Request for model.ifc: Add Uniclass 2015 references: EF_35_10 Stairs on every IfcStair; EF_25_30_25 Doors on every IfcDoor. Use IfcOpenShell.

First a look at what the model holds.

```python
import ifcopenshell

model = ifcopenshell.open("model.ifc")
print(model.schema)
print("classifications:", [c.Name for c in model.by_type("IfcClassification")])
for ifc_class in ("IfcDoor", "IfcRoof", "IfcStair", "IfcWall", "IfcWindow"):
    print(ifc_class, len(model.by_type(ifc_class)))
```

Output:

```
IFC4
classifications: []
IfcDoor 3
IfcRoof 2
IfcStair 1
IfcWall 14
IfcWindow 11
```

```python
import ifcopenshell
import ifcopenshell.api.classification

model = ifcopenshell.open("model.ifc")

system = ifcopenshell.api.classification.add_classification(model, classification="Uniclass 2015")

codes = {
    "IfcStair": ("EF_35_10", "Stairs"),
    "IfcDoor": ("EF_25_30_25", "Doors"),
}
for ifc_class, (code, name) in codes.items():
    products = model.by_type(ifc_class)
    ifcopenshell.api.classification.add_reference(
        model, products=products, classification=system, identification=code, name=name
    )
    print(code, len(products))

model.write("model_edited.ifc")
```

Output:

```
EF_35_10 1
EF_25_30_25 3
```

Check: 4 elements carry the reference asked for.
